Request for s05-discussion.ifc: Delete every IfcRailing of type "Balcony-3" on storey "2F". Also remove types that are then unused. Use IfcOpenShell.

First a look at what the model holds.

```python
import ifcopenshell
import ifcopenshell.util.element

model = ifcopenshell.open("s05-discussion.ifc")
print(model.schema)
storey = next(s for s in model.by_type("IfcBuildingStorey") if s.Name == "2F")
railings = [e for e in ifcopenshell.util.element.get_decomposition(storey) if e.is_a("IfcRailing")]
seen = {}
for e in railings:
    element_type = ifcopenshell.util.element.get_type(e)
    name = element_type.Name if element_type not in (None, e) else None
    seen[name] = seen.get(name, 0) + 1
for name, count in sorted(seen.items(), key=str):
    print(count, "x", name)
```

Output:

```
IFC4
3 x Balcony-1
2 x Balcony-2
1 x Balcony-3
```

```python
import ifcopenshell
import ifcopenshell.api.root
import ifcopenshell.util.element

model = ifcopenshell.open("s05-discussion.ifc")

storey = next(s for s in model.by_type("IfcBuildingStorey") if s.Name == "2F")
railings = [e for e in ifcopenshell.util.element.get_decomposition(storey) if e.is_a("IfcRailing")]
targets = [e for e in railings if (t := ifcopenshell.util.element.get_type(e)) not in (None, e) and t.Name == "Balcony-3"]
types = {ifcopenshell.util.element.get_type(e) for e in targets} - {None, *targets}

for e in targets:
    ifcopenshell.api.root.remove_product(model, product=e)
print(len(targets), "removed")

unused = [t for t in types if not ifcopenshell.util.element.get_types(t)]
for t in unused:
    ifcopenshell.api.root.remove_product(model, product=t)
print(len(unused), "unused types removed")

model.write("s05-discussion-out.ifc")
```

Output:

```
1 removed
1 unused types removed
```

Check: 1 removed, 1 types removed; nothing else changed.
